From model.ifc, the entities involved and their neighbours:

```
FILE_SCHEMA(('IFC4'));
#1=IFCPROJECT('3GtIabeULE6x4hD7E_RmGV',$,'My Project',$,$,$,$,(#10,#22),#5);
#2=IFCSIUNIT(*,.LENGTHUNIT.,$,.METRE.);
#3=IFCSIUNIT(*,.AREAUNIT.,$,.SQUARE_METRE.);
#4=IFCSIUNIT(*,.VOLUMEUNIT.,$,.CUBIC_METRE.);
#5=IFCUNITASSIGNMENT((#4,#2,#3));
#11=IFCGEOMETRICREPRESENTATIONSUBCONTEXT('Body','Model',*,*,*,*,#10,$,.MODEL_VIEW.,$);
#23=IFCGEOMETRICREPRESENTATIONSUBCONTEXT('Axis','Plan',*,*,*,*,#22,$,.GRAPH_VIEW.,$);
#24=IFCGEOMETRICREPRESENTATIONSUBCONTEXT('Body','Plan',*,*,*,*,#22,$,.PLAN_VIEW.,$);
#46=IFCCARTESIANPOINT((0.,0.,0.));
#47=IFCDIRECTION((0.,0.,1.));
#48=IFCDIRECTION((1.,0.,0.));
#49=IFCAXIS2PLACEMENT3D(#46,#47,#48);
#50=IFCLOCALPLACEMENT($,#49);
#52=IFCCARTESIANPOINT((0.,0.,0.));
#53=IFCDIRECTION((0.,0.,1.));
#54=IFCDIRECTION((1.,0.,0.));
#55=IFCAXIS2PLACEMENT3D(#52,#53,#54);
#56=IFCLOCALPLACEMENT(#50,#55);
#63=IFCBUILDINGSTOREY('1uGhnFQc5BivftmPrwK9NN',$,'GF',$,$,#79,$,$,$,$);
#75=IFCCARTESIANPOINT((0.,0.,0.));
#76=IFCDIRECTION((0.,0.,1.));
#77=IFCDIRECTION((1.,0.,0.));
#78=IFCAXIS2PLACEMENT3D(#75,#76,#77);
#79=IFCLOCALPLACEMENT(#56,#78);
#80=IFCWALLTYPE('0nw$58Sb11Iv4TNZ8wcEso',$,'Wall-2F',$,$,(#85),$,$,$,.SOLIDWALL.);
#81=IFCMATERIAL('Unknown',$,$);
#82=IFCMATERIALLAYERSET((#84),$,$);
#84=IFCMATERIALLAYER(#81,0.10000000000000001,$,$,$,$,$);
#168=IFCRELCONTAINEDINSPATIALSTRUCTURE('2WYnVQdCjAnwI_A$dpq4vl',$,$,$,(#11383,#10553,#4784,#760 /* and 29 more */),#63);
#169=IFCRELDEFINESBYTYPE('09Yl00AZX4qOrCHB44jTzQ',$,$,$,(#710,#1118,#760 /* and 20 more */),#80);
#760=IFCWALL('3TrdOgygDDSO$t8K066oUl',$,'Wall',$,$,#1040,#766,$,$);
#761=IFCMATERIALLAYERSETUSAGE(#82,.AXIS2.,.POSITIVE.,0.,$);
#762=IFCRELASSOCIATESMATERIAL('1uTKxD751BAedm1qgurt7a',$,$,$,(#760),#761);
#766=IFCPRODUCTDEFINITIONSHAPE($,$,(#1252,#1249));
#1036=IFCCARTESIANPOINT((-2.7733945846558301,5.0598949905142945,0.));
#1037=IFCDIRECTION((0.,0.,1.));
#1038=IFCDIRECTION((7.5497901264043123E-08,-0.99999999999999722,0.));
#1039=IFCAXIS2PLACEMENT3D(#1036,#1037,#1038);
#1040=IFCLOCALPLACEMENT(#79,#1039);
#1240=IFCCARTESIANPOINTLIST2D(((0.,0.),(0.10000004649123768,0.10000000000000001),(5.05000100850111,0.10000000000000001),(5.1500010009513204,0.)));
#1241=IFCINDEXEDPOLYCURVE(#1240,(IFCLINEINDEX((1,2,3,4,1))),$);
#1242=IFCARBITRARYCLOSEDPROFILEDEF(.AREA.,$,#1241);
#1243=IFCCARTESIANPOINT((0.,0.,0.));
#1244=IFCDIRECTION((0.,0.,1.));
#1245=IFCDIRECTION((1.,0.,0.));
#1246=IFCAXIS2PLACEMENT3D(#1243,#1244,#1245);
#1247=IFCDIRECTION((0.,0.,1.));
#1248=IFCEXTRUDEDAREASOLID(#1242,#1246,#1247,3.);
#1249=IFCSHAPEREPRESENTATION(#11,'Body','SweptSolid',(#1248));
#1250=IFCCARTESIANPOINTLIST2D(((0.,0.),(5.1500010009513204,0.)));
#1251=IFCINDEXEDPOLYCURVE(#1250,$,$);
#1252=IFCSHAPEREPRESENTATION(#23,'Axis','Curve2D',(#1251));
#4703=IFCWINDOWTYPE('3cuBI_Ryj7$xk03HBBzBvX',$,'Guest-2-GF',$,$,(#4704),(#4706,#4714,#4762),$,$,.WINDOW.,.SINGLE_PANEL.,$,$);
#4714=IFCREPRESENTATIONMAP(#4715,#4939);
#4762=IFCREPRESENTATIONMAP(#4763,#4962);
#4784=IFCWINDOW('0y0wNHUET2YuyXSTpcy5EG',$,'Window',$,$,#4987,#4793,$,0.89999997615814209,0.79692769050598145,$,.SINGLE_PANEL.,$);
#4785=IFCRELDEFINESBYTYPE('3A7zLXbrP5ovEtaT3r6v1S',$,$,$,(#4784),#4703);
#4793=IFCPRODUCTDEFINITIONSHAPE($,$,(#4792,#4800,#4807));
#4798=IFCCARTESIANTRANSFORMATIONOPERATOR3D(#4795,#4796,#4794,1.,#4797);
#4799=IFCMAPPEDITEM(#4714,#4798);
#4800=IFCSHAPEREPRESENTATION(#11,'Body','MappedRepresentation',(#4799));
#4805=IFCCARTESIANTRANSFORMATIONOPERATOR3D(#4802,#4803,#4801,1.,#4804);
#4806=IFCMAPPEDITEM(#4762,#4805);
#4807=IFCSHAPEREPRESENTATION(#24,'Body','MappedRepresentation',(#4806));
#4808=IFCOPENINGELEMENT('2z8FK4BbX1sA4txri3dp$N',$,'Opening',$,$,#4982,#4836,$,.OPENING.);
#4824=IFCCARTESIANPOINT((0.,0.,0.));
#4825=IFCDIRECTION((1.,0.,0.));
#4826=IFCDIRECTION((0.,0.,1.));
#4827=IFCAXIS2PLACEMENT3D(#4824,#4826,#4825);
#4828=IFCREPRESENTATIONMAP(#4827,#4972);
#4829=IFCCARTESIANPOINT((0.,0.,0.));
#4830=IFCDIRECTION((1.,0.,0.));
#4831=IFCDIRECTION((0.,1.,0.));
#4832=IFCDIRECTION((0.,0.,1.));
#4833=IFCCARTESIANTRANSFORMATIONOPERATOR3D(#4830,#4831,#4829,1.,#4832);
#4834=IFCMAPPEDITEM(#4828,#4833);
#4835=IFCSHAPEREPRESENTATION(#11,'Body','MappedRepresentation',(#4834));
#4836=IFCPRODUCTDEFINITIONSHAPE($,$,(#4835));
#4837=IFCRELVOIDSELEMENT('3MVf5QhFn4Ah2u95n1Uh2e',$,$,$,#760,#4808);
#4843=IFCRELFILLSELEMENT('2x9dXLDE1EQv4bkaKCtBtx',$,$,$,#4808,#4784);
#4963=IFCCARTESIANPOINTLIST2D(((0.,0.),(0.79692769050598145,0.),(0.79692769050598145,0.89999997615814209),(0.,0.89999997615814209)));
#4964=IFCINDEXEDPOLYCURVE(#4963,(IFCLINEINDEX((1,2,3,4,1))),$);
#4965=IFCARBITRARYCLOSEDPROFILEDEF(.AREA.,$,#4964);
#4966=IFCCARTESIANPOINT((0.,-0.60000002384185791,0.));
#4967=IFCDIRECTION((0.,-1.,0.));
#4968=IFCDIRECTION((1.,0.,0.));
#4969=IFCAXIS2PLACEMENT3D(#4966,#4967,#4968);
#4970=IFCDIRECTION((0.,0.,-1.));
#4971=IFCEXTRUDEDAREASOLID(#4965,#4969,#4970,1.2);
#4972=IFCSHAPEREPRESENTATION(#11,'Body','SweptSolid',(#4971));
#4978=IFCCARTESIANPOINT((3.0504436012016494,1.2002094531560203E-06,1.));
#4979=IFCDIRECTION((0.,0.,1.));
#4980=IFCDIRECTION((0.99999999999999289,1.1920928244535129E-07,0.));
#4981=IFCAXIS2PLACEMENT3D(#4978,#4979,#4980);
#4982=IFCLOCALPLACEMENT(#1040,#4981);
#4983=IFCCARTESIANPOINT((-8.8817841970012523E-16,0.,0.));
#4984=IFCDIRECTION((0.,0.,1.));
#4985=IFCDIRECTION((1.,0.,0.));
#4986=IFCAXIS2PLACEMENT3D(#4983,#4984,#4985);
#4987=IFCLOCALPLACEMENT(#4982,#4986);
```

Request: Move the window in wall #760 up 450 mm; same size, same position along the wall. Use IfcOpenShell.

```python
import numpy as np
import ifcopenshell
import ifcopenshell.api.geometry
import ifcopenshell.util.placement
import ifcopenshell.util.unit

model = ifcopenshell.open("model.ifc")
unit_scale = ifcopenshell.util.unit.calculate_unit_scale(model)

window = model.by_id(4784)
opening = window.FillsVoids[0].RelatingOpeningElement
dz = 0.45

shift = np.array([0.0, 0.0, dz])
# The window is placed relative to its opening, so it follows when the opening moves.
matrix = ifcopenshell.util.placement.get_local_placement(opening.ObjectPlacement)
matrix[:3, 3] += shift
ifcopenshell.api.geometry.edit_object_placement(
    model, product=opening, matrix=matrix, is_si=False, should_transform_children=True
)

print(f"moved by {dz * unit_scale:+.3f} m")

model.write("model_edited.ifc")
```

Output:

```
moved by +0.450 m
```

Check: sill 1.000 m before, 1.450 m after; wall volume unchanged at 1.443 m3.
